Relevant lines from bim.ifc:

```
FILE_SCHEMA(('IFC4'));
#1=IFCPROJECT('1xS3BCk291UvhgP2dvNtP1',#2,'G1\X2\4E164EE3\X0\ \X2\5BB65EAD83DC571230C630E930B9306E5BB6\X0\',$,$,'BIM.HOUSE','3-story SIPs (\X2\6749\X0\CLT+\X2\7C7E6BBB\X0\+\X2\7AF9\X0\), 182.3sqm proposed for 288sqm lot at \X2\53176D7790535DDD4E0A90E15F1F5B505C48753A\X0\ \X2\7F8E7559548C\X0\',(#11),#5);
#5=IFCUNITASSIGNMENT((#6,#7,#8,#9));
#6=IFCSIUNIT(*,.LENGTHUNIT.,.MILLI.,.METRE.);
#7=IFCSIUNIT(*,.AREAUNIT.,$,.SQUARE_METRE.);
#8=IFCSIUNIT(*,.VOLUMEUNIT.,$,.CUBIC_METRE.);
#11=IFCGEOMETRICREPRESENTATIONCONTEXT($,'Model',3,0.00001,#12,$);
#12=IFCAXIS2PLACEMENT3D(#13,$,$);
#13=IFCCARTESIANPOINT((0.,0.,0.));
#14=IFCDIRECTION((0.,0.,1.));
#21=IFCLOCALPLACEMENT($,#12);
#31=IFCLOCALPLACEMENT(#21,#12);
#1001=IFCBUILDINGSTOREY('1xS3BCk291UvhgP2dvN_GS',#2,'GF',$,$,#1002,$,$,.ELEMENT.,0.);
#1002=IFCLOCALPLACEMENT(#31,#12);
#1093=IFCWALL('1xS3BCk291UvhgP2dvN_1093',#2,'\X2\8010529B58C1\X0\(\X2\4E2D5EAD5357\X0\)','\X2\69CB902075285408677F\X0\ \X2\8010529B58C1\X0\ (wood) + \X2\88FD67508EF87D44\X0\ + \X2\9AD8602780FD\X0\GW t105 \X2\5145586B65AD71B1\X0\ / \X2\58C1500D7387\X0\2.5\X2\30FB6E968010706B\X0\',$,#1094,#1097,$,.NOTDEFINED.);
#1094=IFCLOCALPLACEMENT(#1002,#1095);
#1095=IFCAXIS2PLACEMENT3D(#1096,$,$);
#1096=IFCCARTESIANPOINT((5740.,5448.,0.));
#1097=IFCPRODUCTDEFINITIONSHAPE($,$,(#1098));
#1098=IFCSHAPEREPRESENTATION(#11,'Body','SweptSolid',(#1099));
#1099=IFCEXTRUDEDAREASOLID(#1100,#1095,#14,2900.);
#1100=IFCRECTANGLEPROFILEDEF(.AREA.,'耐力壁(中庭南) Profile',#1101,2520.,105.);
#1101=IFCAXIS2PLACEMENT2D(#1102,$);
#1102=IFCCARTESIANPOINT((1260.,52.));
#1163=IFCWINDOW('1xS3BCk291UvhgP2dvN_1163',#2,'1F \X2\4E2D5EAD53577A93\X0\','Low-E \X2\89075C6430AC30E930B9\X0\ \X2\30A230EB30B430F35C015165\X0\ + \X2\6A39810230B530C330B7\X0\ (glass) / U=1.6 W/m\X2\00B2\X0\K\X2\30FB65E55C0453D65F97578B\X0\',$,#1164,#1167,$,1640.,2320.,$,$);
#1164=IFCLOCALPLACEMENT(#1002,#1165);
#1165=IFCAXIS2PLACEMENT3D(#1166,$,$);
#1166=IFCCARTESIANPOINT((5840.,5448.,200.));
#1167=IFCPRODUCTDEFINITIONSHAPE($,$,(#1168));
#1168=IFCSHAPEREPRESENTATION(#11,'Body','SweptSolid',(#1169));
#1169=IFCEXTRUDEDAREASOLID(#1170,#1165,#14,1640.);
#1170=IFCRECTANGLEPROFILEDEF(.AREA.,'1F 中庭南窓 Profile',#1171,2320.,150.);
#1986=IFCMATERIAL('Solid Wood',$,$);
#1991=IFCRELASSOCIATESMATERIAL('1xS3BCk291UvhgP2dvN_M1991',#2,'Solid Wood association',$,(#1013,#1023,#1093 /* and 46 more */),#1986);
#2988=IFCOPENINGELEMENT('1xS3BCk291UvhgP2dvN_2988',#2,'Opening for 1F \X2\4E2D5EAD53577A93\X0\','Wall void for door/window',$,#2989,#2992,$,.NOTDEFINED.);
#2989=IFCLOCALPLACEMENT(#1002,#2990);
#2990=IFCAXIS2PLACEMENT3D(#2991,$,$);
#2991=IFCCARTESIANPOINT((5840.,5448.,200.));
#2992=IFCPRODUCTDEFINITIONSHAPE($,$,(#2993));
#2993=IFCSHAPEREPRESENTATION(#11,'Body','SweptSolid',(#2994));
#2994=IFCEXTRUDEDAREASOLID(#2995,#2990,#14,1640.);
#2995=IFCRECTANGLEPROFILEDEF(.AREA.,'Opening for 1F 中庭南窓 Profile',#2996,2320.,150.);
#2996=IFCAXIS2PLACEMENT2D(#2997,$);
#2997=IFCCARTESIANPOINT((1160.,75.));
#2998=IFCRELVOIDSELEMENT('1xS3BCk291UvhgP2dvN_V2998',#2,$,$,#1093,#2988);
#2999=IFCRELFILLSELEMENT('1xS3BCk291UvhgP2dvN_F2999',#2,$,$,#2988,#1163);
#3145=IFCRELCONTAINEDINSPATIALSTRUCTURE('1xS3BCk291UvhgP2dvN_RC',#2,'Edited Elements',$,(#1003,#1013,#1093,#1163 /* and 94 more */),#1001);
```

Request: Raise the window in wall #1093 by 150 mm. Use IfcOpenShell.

```python
import numpy as np
import ifcopenshell
import ifcopenshell.api.geometry
import ifcopenshell.util.placement
import ifcopenshell.util.unit

model = ifcopenshell.open("bim.ifc")
unit_scale = ifcopenshell.util.unit.calculate_unit_scale(model)

window = model.by_guid("1xS3BCk291UvhgP2dvN_1163")
opening = window.FillsVoids[0].RelatingOpeningElement
dz = 150.0

shift = np.array([0.0, 0.0, dz])
# The window is not placed relative to its opening, so move both.
for product in (opening, window):
    matrix = ifcopenshell.util.placement.get_local_placement(product.ObjectPlacement)
    matrix[:3, 3] += shift
    ifcopenshell.api.geometry.edit_object_placement(model, product=product, matrix=matrix, is_si=False)

print(f"moved by {dz * unit_scale:+.3f} m")

model.write("bim_rev.ifc")
```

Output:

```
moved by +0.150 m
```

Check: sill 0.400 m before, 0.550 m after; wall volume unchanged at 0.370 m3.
